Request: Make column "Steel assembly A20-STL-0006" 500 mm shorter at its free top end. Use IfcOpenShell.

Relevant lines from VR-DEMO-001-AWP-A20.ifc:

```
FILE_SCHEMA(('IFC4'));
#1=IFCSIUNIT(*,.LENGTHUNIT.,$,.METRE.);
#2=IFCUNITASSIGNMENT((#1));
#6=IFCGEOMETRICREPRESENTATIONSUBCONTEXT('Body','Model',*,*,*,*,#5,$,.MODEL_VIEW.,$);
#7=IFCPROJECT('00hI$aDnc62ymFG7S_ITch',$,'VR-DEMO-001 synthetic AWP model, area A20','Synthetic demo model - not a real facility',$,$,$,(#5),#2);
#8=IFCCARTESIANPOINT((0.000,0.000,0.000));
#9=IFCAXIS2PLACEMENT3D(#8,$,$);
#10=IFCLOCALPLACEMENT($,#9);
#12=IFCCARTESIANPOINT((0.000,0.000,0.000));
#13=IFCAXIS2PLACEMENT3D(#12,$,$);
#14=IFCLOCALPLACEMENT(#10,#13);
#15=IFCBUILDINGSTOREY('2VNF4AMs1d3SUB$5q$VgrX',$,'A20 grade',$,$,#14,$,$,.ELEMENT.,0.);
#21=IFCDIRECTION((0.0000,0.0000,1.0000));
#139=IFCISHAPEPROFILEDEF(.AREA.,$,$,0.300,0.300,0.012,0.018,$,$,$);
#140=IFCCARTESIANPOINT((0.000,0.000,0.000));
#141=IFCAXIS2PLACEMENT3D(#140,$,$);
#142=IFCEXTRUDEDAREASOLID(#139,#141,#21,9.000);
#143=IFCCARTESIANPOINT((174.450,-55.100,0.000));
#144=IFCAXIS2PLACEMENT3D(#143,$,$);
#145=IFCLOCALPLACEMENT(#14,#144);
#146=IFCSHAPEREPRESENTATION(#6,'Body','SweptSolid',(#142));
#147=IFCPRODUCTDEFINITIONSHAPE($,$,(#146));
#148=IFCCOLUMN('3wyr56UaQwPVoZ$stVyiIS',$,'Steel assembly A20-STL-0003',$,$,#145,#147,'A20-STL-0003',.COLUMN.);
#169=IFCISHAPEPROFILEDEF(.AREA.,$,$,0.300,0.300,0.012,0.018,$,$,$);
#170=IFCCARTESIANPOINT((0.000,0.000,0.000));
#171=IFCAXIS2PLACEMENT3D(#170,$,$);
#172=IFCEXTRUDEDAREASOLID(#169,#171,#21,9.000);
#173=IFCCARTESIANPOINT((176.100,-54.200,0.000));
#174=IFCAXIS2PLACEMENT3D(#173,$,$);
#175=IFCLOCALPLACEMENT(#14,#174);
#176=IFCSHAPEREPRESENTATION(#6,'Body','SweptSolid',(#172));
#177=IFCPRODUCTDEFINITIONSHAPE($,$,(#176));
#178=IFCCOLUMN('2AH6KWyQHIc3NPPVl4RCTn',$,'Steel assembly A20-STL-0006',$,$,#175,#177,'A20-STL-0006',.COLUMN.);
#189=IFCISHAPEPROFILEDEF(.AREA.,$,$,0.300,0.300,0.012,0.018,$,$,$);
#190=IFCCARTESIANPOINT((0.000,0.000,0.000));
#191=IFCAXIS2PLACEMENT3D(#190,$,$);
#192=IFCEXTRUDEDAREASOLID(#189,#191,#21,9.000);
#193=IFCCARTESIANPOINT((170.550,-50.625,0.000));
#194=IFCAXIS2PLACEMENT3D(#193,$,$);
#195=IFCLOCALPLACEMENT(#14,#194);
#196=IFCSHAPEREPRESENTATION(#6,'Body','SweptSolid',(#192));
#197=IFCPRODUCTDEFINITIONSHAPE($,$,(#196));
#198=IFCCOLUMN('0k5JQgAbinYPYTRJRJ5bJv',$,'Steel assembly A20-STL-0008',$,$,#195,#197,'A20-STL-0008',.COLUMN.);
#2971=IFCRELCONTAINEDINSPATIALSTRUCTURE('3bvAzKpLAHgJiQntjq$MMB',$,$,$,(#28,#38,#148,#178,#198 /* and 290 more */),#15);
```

```python
import ifcopenshell
import ifcopenshell.util.representation
import ifcopenshell.util.unit

model = ifcopenshell.open("VR-DEMO-001-AWP-A20.ifc")
unit_scale = ifcopenshell.util.unit.calculate_unit_scale(model)

member = model.by_guid("2AH6KWyQHIc3NPPVl4RCTn")
change = -0.5 / unit_scale

# The extrusion runs towards the end named, so only its depth changes.
body = ifcopenshell.util.representation.get_representation(member, "Model", "Body")
solid = body.Items[0]
old_length = solid.Depth
solid.Depth += change

print(f"length {old_length:g} -> {solid.Depth:g}")

model.write("VR-DEMO-001-AWP-A20_edited.ifc")
```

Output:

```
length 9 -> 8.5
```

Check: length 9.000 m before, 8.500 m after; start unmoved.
